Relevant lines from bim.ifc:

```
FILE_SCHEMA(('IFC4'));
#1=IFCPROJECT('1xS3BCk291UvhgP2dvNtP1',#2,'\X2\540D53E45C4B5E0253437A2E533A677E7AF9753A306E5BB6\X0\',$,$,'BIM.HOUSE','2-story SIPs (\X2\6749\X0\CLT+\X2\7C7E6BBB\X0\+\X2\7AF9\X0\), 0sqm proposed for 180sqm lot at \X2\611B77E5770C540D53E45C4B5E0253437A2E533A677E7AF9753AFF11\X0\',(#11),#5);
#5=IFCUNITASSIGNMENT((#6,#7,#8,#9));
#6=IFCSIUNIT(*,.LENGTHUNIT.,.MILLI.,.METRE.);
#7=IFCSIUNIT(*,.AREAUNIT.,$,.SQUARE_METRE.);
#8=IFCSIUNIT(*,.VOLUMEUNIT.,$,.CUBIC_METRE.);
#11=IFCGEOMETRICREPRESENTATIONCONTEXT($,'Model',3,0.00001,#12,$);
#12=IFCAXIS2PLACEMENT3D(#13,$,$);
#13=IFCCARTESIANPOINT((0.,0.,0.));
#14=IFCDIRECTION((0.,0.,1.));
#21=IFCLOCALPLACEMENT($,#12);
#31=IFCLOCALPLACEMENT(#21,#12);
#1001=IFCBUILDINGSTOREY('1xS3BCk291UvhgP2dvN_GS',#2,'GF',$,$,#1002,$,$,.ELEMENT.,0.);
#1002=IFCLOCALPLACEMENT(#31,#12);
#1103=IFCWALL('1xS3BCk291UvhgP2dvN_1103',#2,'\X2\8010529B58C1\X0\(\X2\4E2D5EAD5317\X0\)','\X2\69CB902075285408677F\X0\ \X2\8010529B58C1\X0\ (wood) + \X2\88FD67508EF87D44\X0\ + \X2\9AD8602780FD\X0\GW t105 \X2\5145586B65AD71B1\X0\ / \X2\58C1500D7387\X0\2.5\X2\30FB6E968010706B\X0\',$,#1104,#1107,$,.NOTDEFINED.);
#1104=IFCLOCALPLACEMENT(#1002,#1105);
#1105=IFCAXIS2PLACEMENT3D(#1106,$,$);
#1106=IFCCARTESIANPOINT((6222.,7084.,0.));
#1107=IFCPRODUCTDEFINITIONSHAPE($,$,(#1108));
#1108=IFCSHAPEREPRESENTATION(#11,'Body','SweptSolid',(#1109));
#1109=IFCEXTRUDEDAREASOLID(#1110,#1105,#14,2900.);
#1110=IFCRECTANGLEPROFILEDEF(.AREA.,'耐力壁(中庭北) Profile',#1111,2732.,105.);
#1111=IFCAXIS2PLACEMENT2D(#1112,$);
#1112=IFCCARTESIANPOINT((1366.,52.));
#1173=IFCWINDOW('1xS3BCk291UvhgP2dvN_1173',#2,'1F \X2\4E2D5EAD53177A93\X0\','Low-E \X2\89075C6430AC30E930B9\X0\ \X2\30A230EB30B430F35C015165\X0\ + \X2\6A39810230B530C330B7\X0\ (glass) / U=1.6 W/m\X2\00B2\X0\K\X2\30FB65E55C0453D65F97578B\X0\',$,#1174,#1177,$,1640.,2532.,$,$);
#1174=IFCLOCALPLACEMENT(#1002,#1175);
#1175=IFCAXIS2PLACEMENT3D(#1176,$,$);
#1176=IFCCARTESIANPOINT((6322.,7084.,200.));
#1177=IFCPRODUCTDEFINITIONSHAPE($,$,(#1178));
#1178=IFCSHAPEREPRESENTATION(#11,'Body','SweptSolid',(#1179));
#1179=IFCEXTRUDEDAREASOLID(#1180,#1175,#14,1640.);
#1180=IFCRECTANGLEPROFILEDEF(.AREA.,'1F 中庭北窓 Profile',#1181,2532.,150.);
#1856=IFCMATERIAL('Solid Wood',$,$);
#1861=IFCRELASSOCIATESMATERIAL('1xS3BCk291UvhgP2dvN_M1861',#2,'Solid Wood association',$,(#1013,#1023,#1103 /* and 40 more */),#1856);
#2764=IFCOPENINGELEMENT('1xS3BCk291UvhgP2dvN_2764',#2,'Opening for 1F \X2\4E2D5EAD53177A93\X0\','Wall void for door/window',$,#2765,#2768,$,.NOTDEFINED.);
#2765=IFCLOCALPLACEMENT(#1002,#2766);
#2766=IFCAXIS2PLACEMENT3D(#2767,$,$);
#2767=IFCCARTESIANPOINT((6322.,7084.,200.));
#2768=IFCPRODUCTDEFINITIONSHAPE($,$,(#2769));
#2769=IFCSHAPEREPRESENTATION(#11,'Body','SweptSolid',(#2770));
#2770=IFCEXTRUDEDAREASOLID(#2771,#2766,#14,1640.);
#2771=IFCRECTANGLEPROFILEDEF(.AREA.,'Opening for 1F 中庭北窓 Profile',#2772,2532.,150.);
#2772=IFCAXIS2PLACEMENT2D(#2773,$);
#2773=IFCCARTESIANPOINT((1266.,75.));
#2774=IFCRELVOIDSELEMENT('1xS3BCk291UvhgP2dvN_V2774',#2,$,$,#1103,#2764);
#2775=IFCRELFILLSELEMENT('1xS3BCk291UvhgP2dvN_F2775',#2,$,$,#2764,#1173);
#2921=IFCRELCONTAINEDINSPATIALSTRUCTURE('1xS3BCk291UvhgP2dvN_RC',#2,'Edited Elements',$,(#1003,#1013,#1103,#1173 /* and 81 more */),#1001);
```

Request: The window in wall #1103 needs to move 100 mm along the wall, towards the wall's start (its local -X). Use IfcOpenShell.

```python
import ifcopenshell
import ifcopenshell.api.geometry
import ifcopenshell.util.placement
import ifcopenshell.util.unit

model = ifcopenshell.open("bim.ifc")
unit_scale = ifcopenshell.util.unit.calculate_unit_scale(model)

window = model.by_guid("1xS3BCk291UvhgP2dvN_1173")
opening = window.FillsVoids[0].RelatingOpeningElement
wall = opening.VoidsElements[0].RelatingBuildingElement

wall_matrix = ifcopenshell.util.placement.get_local_placement(wall.ObjectPlacement)
shift = wall_matrix[:3, 0] * -0.1 / unit_scale
before = ifcopenshell.util.placement.get_local_placement(window.ObjectPlacement)[:3, 3].copy()

# The window is not placed relative to its opening, so move both.
for product in (opening, window):
    matrix = ifcopenshell.util.placement.get_local_placement(product.ObjectPlacement)
    matrix[:3, 3] += shift
    ifcopenshell.api.geometry.edit_object_placement(model, product=product, matrix=matrix, is_si=False)

after = ifcopenshell.util.placement.get_local_placement(window.ObjectPlacement)[:3, 3]
print("window moved by", (after - before).round(3) + 0.0)

model.write("bim_rev.ifc")
```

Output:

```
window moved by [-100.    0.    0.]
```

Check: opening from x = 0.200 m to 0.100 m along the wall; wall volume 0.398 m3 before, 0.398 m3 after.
